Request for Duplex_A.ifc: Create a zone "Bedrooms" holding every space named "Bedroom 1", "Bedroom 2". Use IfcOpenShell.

First a look at what the model holds.

```python
import ifcopenshell

model = ifcopenshell.open("Duplex_A.ifc")
print(model.schema)
seen = {}
for space in model.by_type("IfcSpace"):
    seen[space.LongName] = seen.get(space.LongName, 0) + 1
for name, count in sorted(seen.items(), key=str):
    print(count, "x", name)
print("zones:", [z.Name for z in model.by_type("IfcZone")][:20])
```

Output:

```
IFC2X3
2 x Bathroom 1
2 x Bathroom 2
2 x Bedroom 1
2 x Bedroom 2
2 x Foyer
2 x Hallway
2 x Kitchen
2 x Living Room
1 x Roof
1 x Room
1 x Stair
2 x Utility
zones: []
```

```python
import ifcopenshell
import ifcopenshell.api.group
import ifcopenshell.api.root

model = ifcopenshell.open("Duplex_A.ifc")

names = {"Bedroom 1", "Bedroom 2"}
spaces = [s for s in model.by_type("IfcSpace") if s.LongName in names]

zone = ifcopenshell.api.root.create_entity(model, ifc_class="IfcZone", name="Bedrooms")
ifcopenshell.api.group.assign_group(model, products=spaces, group=zone)
print(len(spaces), "spaces in", zone.Name)

model.write("Duplex_A_edited.ifc")
```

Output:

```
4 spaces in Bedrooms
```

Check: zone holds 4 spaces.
